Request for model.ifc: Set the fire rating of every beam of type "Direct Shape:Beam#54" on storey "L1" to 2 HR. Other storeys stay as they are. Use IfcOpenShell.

First a look at what the model holds.

```python
import ifcopenshell
import ifcopenshell.util.element

model = ifcopenshell.open("model.ifc")
print(model.schema)
storey = next(s for s in model.by_type("IfcBuildingStorey") if s.Name == "L1")
beams = [e for e in ifcopenshell.util.element.get_decomposition(storey) if e.is_a("IfcBeam")]
seen = {}
for e in beams:
    element_type = ifcopenshell.util.element.get_type(e)
    key = (element_type.Name if element_type != e and element_type else None, ifcopenshell.util.element.get_pset(e, "Pset_BeamCommon", "FireRating"))
    seen[key] = seen.get(key, 0) + 1
for (name, value), count in sorted(seen.items(), key=str):
    print(count, "x", name, "|", value)
```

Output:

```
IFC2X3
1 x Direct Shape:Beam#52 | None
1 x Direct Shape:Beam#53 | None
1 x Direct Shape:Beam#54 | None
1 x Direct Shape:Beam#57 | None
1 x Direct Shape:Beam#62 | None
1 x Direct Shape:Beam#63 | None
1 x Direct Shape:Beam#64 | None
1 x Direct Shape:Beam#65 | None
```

```python
import ifcopenshell
import ifcopenshell.api.pset
import ifcopenshell.util.element

model = ifcopenshell.open("model.ifc")

storey = next(s for s in model.by_type("IfcBuildingStorey") if s.Name == "L1")
beams = [e for e in ifcopenshell.util.element.get_decomposition(storey) if e.is_a("IfcBeam")]

count = 0
for e in beams:
    element_type = ifcopenshell.util.element.get_type(e)
    if element_type in (None, e) or element_type.Name != "Direct Shape:Beam#54":
        continue
    # add_pset returns the element's existing set when there is one.
    pset = ifcopenshell.api.pset.add_pset(model, product=e, name="Pset_BeamCommon")
    ifcopenshell.api.pset.edit_pset(model, pset=pset, properties={"FireRating": "2 HR"})
    count += 1

print(count, "beams updated")

model.write("model-out.ifc")
```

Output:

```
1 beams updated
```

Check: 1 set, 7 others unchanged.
